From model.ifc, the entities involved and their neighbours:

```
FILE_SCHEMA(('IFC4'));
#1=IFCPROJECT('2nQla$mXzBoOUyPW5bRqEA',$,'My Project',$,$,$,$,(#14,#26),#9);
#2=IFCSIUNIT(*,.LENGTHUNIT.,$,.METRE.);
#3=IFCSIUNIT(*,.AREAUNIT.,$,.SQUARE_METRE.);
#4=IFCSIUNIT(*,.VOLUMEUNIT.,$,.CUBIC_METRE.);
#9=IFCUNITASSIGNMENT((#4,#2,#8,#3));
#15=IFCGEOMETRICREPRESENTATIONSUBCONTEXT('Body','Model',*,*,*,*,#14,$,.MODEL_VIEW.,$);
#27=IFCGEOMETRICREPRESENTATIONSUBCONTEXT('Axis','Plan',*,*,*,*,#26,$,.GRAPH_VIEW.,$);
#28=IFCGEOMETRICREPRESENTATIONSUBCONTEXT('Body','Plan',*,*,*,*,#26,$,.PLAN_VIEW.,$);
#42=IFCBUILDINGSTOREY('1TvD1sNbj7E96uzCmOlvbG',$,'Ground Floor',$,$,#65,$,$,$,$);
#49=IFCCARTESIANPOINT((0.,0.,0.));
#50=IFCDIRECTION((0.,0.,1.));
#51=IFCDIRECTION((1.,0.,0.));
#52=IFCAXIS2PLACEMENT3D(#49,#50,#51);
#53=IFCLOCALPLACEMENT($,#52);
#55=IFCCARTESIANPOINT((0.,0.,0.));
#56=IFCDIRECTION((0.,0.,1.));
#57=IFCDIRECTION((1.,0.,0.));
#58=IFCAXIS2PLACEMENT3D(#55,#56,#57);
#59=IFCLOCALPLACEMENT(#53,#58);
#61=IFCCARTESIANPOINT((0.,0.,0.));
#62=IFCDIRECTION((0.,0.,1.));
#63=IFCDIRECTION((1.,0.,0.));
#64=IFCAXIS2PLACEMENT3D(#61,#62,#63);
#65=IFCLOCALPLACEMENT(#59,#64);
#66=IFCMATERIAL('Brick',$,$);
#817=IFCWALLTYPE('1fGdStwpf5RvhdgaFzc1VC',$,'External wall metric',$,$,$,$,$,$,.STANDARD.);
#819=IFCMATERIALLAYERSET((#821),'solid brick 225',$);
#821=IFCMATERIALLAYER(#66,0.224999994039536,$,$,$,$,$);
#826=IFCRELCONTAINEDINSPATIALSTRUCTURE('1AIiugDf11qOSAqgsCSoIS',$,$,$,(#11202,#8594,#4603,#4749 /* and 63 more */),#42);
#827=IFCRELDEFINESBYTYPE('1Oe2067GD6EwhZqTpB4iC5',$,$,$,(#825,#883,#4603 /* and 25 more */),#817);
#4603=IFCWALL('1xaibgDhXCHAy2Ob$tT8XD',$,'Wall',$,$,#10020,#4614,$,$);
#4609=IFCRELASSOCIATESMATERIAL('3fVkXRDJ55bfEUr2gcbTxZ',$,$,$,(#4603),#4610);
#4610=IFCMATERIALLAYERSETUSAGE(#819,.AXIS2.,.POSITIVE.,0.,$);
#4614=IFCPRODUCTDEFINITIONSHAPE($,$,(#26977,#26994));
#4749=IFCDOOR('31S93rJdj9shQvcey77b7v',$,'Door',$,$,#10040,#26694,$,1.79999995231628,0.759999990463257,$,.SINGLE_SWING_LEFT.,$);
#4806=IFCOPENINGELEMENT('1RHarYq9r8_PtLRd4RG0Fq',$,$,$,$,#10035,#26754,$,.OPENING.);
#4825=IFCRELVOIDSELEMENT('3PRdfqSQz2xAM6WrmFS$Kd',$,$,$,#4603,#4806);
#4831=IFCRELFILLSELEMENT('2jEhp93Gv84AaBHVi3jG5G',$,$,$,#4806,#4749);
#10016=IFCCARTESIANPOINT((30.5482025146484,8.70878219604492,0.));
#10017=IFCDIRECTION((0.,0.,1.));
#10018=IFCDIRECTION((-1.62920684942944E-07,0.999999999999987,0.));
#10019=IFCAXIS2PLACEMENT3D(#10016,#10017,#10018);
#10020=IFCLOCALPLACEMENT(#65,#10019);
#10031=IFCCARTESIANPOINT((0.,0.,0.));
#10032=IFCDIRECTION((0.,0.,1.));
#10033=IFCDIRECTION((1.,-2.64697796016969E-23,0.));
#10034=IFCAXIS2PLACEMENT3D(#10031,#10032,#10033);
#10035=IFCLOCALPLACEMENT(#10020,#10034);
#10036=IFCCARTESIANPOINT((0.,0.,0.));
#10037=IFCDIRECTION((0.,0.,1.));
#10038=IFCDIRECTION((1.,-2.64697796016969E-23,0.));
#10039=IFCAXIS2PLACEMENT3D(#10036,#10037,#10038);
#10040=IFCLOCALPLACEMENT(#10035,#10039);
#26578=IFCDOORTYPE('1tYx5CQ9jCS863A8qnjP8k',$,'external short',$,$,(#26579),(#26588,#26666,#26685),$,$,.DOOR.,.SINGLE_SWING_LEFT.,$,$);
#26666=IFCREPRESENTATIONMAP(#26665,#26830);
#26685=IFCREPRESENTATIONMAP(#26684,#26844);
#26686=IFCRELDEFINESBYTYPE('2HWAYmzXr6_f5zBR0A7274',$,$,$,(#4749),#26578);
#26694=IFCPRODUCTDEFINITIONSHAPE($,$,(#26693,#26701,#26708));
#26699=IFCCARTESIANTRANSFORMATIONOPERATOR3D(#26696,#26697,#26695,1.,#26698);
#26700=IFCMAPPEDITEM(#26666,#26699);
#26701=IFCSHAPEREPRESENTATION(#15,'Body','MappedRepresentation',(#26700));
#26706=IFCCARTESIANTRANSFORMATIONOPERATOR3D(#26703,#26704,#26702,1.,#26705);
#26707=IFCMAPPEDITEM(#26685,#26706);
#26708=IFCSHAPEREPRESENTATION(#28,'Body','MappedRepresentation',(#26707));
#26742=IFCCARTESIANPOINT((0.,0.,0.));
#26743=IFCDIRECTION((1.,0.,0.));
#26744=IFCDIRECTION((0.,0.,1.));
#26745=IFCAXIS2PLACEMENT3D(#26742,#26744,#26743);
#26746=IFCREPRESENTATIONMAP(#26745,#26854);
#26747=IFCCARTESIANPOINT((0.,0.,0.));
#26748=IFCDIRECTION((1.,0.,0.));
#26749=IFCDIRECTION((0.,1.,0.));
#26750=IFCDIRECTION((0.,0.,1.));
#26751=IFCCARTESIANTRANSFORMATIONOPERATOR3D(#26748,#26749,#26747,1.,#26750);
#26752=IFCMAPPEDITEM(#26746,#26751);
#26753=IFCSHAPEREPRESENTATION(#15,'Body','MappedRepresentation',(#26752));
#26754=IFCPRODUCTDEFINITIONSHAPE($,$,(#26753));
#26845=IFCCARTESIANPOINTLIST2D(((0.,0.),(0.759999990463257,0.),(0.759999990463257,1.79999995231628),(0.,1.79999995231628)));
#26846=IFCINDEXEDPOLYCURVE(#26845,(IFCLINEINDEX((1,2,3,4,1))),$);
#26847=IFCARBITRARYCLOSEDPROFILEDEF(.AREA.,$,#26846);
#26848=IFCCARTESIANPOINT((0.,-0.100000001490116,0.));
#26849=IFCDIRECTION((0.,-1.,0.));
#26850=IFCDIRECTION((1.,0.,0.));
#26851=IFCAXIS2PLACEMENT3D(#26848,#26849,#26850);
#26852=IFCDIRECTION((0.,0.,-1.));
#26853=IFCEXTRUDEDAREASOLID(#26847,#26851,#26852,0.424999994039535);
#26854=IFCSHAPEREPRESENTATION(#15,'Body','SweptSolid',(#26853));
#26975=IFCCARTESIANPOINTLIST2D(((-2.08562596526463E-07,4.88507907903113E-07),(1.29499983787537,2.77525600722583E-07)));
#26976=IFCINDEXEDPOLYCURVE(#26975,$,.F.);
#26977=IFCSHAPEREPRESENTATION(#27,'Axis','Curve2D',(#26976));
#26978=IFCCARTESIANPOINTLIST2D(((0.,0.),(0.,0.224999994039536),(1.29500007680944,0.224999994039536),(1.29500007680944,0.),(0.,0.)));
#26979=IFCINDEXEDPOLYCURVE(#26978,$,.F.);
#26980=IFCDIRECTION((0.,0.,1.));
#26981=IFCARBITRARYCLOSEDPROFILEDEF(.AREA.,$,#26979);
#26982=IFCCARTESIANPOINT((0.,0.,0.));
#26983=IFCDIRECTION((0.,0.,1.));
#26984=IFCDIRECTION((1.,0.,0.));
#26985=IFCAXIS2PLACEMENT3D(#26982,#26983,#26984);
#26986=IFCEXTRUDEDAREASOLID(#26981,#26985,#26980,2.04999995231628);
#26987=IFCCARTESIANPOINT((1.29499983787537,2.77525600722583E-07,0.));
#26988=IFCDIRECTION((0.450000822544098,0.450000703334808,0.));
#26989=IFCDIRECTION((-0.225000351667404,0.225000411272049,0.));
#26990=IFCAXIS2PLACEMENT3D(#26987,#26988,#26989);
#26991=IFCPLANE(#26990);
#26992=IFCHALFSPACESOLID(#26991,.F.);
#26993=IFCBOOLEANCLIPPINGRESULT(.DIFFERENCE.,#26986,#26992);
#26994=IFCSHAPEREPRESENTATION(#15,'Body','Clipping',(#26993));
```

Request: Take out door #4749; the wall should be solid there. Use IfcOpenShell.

```python
import ifcopenshell
import ifcopenshell.api.feature
import ifcopenshell.api.root
import ifcopenshell.geom
import ifcopenshell.util.shape

model = ifcopenshell.open("model.ifc")
settings = ifcopenshell.geom.settings()


def volume(element):
    """Net volume in cubic metres, openings subtracted."""
    shape = ifcopenshell.geom.create_shape(settings, element)
    return ifcopenshell.util.shape.get_volume(shape.geometry)


door = model.by_guid("31S93rJdj9shQvcey77b7v")
opening = door.FillsVoids[0].RelatingOpeningElement
wall = opening.VoidsElements[0].RelatingBuildingElement
before = volume(wall)

ifcopenshell.api.root.remove_product(model, product=door)
ifcopenshell.api.feature.remove_feature(model, feature=opening)

after = volume(wall)

print(f"wall volume {before:.3f} -> {after:.3f} m3")

model.write("model_v2.ifc")
```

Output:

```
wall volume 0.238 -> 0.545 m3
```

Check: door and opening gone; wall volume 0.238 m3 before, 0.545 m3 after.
